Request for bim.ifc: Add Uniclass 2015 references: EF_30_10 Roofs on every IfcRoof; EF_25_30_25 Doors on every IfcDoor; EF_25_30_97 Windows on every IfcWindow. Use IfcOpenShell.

First a look at what the model holds.

```python
import ifcopenshell

model = ifcopenshell.open("bim.ifc")
print(model.schema)
print("classifications:", [c.Name for c in model.by_type("IfcClassification")])
for ifc_class in ("IfcDoor", "IfcRoof", "IfcStair", "IfcWall", "IfcWindow"):
    print(ifc_class, len(model.by_type(ifc_class)))
```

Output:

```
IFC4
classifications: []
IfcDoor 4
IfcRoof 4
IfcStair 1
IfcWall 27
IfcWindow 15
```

```python
import ifcopenshell
import ifcopenshell.api.classification

model = ifcopenshell.open("bim.ifc")

system = ifcopenshell.api.classification.add_classification(model, classification="Uniclass 2015")

codes = {
    "IfcRoof": ("EF_30_10", "Roofs"),
    "IfcDoor": ("EF_25_30_25", "Doors"),
    "IfcWindow": ("EF_25_30_97", "Windows"),
}
for ifc_class, (code, name) in codes.items():
    products = model.by_type(ifc_class)
    ifcopenshell.api.classification.add_reference(
        model, products=products, classification=system, identification=code, name=name
    )
    print(code, len(products))

model.write("bim-out.ifc")
```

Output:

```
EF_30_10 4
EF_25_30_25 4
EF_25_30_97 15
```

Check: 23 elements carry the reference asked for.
